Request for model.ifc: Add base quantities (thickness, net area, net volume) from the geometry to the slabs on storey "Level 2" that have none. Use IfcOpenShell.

First a look at what the model holds.

```python
import ifcopenshell
import ifcopenshell.util.element
import ifcopenshell.util.unit

model = ifcopenshell.open("model.ifc")
print(model.schema)
for unit_type in ("LENGTHUNIT", "AREAUNIT", "VOLUMEUNIT"):
    print(unit_type, ifcopenshell.util.unit.calculate_unit_scale(model, unit_type))
storey = next(s for s in model.by_type("IfcBuildingStorey") if s.Name == "Level 2")
slabs = [e for e in ifcopenshell.util.element.get_decomposition(storey) if e.is_a("IfcSlab")]
for e in sorted(slabs, key=lambda e: e.id()):
    print(e.id(), e.is_a(), e.Name, list(ifcopenshell.util.element.get_psets(e, qtos_only=True)), sep=" | ")
```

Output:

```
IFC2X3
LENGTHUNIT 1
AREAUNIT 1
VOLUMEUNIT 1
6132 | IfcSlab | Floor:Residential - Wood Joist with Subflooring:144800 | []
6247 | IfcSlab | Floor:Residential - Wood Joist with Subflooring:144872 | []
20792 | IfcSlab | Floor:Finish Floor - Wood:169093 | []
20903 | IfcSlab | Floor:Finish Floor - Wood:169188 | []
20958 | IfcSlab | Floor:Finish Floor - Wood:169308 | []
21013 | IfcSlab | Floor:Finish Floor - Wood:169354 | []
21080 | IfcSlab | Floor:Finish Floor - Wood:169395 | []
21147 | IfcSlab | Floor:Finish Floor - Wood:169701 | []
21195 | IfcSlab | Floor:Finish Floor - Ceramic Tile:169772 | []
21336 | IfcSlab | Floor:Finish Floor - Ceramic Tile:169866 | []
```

```python
import ifcopenshell
import ifcopenshell.api.pset
import ifcopenshell.geom
import ifcopenshell.util.element
import ifcopenshell.util.shape
import ifcopenshell.util.unit

model = ifcopenshell.open("model.ifc")
unit_scale = ifcopenshell.util.unit.calculate_unit_scale(model)
area_scale = ifcopenshell.util.unit.calculate_unit_scale(model, "AREAUNIT")
volume_scale = ifcopenshell.util.unit.calculate_unit_scale(model, "VOLUMEUNIT")
settings = ifcopenshell.geom.settings()

storey = next(s for s in model.by_type("IfcBuildingStorey") if s.Name == "Level 2")
slabs = [e for e in ifcopenshell.util.element.get_decomposition(storey) if e.is_a("IfcSlab")]

for e in sorted(slabs, key=lambda e: e.id()):
    if ifcopenshell.util.element.get_psets(e, qtos_only=True, should_inherit=False):
        continue
    # Geometry comes back in metres, in the element's own axes.
    shape = ifcopenshell.geom.create_shape(settings, e)
    values = {
        "Width": ifcopenshell.util.shape.get_z(shape.geometry) / unit_scale,
        "NetArea": ifcopenshell.util.shape.get_footprint_area(shape.geometry) / area_scale,
        "NetVolume": ifcopenshell.util.shape.get_volume(shape.geometry) / volume_scale,
    }
    qto = ifcopenshell.api.pset.add_qto(model, product=e, name="BaseQuantities")
    ifcopenshell.api.pset.edit_qto(model, qto=qto, properties=values)
    print(e.id(), {k: round(v, 3) for k, v in values.items()})

model.write("model_rev.ifc")
```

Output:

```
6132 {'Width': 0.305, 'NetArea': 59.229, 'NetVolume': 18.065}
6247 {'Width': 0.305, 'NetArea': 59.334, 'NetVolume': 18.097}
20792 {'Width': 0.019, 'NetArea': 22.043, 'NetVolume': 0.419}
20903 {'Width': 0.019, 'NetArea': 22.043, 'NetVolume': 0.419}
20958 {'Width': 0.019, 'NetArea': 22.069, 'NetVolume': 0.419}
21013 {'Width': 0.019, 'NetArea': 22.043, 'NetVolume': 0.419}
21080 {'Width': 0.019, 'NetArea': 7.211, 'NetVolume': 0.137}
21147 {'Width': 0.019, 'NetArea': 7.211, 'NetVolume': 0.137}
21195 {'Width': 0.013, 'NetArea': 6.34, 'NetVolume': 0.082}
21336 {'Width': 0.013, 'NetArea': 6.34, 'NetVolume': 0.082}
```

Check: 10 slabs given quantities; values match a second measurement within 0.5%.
